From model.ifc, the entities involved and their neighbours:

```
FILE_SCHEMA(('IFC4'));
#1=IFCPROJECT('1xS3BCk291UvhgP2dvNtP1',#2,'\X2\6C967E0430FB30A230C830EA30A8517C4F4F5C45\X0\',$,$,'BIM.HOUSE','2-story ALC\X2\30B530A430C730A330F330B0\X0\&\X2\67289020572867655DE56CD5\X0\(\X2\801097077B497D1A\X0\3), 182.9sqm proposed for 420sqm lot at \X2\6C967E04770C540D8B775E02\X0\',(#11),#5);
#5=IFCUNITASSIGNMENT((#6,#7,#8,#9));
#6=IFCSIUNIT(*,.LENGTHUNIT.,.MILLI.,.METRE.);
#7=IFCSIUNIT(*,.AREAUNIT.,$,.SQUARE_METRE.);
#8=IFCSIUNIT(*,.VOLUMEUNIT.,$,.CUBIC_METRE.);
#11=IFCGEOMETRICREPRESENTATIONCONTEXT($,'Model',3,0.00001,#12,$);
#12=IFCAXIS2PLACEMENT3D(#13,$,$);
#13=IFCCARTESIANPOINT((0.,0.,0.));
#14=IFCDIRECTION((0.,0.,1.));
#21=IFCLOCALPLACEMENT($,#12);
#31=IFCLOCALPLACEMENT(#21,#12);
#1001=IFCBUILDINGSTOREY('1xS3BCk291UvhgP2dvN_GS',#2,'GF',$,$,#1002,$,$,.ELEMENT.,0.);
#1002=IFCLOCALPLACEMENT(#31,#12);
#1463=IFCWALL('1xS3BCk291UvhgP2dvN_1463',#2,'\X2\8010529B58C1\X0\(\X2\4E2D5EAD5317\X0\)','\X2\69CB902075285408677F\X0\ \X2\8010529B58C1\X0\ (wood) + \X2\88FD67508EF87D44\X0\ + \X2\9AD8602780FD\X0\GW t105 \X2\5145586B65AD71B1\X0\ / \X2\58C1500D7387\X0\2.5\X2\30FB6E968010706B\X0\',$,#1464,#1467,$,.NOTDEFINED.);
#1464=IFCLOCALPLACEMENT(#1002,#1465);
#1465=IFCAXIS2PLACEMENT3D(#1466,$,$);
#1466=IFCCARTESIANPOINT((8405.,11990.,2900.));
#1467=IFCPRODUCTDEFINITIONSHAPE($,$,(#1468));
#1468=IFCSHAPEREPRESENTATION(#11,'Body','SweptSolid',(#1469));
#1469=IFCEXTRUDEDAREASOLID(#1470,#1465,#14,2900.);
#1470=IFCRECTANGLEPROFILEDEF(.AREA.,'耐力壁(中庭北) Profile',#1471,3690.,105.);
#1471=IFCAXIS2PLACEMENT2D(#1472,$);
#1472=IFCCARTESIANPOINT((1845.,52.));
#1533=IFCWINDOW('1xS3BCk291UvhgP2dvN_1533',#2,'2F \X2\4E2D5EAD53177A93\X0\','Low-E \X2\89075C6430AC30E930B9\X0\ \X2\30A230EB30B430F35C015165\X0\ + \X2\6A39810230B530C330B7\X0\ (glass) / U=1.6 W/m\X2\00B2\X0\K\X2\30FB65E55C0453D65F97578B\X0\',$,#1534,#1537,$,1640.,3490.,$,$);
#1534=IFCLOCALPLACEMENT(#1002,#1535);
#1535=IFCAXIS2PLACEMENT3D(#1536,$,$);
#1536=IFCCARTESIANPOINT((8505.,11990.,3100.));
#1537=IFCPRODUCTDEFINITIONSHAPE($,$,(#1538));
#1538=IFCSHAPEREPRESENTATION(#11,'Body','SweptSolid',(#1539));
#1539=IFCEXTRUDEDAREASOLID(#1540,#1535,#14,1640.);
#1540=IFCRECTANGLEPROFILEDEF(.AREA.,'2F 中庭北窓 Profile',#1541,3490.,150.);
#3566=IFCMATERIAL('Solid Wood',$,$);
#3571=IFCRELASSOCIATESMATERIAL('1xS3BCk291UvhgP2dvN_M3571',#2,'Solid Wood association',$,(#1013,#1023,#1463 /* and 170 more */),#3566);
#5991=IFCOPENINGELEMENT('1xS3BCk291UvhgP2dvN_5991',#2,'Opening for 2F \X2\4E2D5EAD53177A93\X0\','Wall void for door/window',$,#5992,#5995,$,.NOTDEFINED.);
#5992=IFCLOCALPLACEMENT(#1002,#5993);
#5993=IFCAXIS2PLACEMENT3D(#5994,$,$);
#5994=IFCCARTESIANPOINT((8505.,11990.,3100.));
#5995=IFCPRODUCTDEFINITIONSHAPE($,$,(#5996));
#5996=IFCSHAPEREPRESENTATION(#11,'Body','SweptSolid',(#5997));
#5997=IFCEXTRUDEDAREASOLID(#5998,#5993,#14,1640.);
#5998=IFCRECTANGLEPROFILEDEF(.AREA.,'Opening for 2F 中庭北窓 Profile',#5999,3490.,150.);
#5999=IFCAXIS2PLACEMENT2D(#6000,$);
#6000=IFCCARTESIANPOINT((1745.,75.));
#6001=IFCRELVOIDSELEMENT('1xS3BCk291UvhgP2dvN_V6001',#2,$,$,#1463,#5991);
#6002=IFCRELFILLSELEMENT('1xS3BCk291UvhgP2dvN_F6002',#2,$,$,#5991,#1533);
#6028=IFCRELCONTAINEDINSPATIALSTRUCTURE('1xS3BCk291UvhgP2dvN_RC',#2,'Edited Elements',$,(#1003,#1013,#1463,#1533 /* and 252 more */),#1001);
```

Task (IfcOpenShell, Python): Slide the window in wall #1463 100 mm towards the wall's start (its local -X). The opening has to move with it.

```python
import ifcopenshell
import ifcopenshell.api.geometry
import ifcopenshell.util.placement
import ifcopenshell.util.unit

model = ifcopenshell.open("model.ifc")
unit_scale = ifcopenshell.util.unit.calculate_unit_scale(model)

window = model.by_id(1533)
opening = window.FillsVoids[0].RelatingOpeningElement
wall = opening.VoidsElements[0].RelatingBuildingElement

wall_matrix = ifcopenshell.util.placement.get_local_placement(wall.ObjectPlacement)
shift = wall_matrix[:3, 0] * -0.1 / unit_scale
before = ifcopenshell.util.placement.get_local_placement(window.ObjectPlacement)[:3, 3].copy()

# The window is not placed relative to its opening, so move both.
for product in (opening, window):
    matrix = ifcopenshell.util.placement.get_local_placement(product.ObjectPlacement)
    matrix[:3, 3] += shift
    ifcopenshell.api.geometry.edit_object_placement(model, product=product, matrix=matrix, is_si=False)

after = ifcopenshell.util.placement.get_local_placement(window.ObjectPlacement)[:3, 3]
print("window moved by", (after - before).round(3) + 0.0)

model.write("model_v2.ifc")
```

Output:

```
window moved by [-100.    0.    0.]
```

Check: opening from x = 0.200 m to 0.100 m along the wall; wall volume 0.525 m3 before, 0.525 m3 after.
